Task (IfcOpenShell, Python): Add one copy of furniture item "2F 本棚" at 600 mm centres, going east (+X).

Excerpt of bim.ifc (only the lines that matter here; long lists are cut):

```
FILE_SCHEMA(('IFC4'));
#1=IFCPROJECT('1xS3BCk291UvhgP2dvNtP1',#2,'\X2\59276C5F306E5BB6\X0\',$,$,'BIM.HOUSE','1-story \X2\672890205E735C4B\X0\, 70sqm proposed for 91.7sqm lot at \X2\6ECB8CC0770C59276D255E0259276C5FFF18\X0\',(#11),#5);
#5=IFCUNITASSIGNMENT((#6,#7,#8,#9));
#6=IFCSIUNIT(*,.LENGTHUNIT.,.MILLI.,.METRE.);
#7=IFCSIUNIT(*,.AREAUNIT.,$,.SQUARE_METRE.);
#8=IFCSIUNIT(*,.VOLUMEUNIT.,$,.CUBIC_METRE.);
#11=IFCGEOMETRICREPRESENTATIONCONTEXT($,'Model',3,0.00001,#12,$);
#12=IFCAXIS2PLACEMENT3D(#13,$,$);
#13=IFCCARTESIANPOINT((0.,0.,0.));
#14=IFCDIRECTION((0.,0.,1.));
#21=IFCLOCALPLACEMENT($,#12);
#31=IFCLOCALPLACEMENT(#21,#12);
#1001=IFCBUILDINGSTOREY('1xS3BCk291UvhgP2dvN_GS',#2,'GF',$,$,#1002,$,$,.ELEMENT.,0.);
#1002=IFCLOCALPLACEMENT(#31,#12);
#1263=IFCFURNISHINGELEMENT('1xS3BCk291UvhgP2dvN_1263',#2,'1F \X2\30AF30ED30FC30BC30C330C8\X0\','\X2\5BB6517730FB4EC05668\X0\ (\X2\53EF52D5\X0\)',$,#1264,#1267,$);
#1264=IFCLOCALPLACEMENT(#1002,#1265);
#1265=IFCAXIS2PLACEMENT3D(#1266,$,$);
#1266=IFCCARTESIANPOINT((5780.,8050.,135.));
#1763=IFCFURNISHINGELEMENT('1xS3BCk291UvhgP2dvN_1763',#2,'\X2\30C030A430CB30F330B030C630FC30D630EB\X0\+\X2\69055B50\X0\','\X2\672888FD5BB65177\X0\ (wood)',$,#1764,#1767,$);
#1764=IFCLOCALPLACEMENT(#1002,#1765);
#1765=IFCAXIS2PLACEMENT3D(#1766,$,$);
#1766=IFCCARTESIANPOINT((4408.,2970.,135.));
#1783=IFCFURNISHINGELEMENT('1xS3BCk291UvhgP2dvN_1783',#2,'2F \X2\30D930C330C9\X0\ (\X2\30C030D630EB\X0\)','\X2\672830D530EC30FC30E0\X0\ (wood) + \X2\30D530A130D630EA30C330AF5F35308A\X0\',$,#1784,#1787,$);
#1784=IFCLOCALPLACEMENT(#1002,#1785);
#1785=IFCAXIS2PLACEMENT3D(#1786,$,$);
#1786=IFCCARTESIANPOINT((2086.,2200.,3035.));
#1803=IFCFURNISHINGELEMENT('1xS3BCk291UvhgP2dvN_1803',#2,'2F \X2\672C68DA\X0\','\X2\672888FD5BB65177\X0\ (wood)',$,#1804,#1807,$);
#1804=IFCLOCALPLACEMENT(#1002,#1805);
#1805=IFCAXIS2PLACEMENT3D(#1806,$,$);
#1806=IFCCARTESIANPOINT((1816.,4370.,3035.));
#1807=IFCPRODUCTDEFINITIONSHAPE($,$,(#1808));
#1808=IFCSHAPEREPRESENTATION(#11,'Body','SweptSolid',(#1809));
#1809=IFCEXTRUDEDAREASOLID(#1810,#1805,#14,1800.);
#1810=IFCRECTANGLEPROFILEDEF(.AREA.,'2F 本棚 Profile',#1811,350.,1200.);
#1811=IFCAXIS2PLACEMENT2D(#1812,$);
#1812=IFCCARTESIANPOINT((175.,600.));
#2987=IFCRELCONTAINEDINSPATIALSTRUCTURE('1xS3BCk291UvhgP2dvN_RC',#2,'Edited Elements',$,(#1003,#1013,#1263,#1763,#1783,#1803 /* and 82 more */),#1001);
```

```python
import numpy as np
import ifcopenshell
import ifcopenshell.api.geometry
import ifcopenshell.api.root
import ifcopenshell.util.element
import ifcopenshell.util.placement
import ifcopenshell.util.unit

model = ifcopenshell.open("bim.ifc")
unit_scale = ifcopenshell.util.unit.calculate_unit_scale(model)


def reuse_history(source, copy):
    """copy_class also copies each property set's owner history, people and application; keep the originals."""
    for rel in copy.IsDefinedBy:
        if rel.is_a("IfcRelDefinesByProperties") and (history := rel.RelatingPropertyDefinition.OwnerHistory):
            rel.RelatingPropertyDefinition.OwnerHistory = source.OwnerHistory
            ifcopenshell.util.element.remove_deep2(model, history)


source = model.by_guid("1xS3BCk291UvhgP2dvN_1803")
base = ifcopenshell.util.placement.get_local_placement(source.ObjectPlacement)
step = np.array([1.0, 0.0, 0.0]) * 0.6 / unit_scale

for i in range(1, 2):
    copy = ifcopenshell.api.root.copy_class(model, product=source)
    copy.Representation = ifcopenshell.util.element.copy_deep(
        model, source.Representation, exclude=["IfcGeometricRepresentationContext", "IfcRepresentationMap"]
    )
    reuse_history(source, copy)
    matrix = base.copy()
    matrix[:3, 3] += i * step
    print("added at", matrix[:3, 3].round(3) + 0.0)
    ifcopenshell.api.geometry.edit_object_placement(model, product=copy, matrix=matrix, is_si=False)

model.write("bim_updated.ifc")
```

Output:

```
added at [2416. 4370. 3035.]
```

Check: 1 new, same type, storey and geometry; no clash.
